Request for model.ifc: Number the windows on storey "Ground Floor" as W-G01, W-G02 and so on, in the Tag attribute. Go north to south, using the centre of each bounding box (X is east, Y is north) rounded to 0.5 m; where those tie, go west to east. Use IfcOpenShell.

First a look at what the model holds.

```python
import ifcopenshell
import ifcopenshell.util.element
import ifcopenshell.util.placement

model = ifcopenshell.open("model.ifc")
print(model.schema)
storey = next(s for s in model.by_type("IfcBuildingStorey") if s.Name == "Ground Floor")
windows = [e for e in ifcopenshell.util.element.get_decomposition(storey) if e.is_a("IfcWindow")]
for e in sorted(windows, key=lambda e: e.id()):
    origin = ifcopenshell.util.placement.get_local_placement(e.ObjectPlacement)[:3, 3]
    print(e.id(), e.Tag, e.Name, origin.round(2) + 0.0, sep=" | ")
```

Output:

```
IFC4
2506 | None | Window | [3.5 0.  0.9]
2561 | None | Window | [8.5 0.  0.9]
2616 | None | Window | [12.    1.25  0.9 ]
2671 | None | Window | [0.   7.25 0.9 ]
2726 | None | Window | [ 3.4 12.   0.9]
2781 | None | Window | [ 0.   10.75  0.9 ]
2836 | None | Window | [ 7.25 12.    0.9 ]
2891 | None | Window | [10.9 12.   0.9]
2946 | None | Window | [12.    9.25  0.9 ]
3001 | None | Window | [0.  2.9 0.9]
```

```python
import ifcopenshell
import ifcopenshell.geom
import ifcopenshell.util.element
import ifcopenshell.util.shape

model = ifcopenshell.open("model.ifc")
settings = ifcopenshell.geom.settings()
settings.set("use-world-coords", True)


def centre(element):
    shape = ifcopenshell.geom.create_shape(settings, element)
    return ifcopenshell.util.shape.get_bbox_centroid(shape.geometry)


storey = next(s for s in model.by_type("IfcBuildingStorey") if s.Name == "Ground Floor")
windows = [e for e in ifcopenshell.util.element.get_decomposition(storey) if e.is_a("IfcWindow")]

# Insertion points can sit at a corner or the storey origin, so sort by the geometry (in metres).
centres = {e: centre(e) for e in windows}
windows.sort(key=lambda e: (-round(centres[e][1] / 0.5), centres[e][0]))

for i, e in enumerate(windows, start=1):
    number = f"W-G{i:02d}"
    e.Tag = number
    print(e.id(), number)

model.write("model-out.ifc")
```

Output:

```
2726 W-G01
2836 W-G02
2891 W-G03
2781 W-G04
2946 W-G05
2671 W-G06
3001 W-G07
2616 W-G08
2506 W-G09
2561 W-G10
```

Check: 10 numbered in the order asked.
